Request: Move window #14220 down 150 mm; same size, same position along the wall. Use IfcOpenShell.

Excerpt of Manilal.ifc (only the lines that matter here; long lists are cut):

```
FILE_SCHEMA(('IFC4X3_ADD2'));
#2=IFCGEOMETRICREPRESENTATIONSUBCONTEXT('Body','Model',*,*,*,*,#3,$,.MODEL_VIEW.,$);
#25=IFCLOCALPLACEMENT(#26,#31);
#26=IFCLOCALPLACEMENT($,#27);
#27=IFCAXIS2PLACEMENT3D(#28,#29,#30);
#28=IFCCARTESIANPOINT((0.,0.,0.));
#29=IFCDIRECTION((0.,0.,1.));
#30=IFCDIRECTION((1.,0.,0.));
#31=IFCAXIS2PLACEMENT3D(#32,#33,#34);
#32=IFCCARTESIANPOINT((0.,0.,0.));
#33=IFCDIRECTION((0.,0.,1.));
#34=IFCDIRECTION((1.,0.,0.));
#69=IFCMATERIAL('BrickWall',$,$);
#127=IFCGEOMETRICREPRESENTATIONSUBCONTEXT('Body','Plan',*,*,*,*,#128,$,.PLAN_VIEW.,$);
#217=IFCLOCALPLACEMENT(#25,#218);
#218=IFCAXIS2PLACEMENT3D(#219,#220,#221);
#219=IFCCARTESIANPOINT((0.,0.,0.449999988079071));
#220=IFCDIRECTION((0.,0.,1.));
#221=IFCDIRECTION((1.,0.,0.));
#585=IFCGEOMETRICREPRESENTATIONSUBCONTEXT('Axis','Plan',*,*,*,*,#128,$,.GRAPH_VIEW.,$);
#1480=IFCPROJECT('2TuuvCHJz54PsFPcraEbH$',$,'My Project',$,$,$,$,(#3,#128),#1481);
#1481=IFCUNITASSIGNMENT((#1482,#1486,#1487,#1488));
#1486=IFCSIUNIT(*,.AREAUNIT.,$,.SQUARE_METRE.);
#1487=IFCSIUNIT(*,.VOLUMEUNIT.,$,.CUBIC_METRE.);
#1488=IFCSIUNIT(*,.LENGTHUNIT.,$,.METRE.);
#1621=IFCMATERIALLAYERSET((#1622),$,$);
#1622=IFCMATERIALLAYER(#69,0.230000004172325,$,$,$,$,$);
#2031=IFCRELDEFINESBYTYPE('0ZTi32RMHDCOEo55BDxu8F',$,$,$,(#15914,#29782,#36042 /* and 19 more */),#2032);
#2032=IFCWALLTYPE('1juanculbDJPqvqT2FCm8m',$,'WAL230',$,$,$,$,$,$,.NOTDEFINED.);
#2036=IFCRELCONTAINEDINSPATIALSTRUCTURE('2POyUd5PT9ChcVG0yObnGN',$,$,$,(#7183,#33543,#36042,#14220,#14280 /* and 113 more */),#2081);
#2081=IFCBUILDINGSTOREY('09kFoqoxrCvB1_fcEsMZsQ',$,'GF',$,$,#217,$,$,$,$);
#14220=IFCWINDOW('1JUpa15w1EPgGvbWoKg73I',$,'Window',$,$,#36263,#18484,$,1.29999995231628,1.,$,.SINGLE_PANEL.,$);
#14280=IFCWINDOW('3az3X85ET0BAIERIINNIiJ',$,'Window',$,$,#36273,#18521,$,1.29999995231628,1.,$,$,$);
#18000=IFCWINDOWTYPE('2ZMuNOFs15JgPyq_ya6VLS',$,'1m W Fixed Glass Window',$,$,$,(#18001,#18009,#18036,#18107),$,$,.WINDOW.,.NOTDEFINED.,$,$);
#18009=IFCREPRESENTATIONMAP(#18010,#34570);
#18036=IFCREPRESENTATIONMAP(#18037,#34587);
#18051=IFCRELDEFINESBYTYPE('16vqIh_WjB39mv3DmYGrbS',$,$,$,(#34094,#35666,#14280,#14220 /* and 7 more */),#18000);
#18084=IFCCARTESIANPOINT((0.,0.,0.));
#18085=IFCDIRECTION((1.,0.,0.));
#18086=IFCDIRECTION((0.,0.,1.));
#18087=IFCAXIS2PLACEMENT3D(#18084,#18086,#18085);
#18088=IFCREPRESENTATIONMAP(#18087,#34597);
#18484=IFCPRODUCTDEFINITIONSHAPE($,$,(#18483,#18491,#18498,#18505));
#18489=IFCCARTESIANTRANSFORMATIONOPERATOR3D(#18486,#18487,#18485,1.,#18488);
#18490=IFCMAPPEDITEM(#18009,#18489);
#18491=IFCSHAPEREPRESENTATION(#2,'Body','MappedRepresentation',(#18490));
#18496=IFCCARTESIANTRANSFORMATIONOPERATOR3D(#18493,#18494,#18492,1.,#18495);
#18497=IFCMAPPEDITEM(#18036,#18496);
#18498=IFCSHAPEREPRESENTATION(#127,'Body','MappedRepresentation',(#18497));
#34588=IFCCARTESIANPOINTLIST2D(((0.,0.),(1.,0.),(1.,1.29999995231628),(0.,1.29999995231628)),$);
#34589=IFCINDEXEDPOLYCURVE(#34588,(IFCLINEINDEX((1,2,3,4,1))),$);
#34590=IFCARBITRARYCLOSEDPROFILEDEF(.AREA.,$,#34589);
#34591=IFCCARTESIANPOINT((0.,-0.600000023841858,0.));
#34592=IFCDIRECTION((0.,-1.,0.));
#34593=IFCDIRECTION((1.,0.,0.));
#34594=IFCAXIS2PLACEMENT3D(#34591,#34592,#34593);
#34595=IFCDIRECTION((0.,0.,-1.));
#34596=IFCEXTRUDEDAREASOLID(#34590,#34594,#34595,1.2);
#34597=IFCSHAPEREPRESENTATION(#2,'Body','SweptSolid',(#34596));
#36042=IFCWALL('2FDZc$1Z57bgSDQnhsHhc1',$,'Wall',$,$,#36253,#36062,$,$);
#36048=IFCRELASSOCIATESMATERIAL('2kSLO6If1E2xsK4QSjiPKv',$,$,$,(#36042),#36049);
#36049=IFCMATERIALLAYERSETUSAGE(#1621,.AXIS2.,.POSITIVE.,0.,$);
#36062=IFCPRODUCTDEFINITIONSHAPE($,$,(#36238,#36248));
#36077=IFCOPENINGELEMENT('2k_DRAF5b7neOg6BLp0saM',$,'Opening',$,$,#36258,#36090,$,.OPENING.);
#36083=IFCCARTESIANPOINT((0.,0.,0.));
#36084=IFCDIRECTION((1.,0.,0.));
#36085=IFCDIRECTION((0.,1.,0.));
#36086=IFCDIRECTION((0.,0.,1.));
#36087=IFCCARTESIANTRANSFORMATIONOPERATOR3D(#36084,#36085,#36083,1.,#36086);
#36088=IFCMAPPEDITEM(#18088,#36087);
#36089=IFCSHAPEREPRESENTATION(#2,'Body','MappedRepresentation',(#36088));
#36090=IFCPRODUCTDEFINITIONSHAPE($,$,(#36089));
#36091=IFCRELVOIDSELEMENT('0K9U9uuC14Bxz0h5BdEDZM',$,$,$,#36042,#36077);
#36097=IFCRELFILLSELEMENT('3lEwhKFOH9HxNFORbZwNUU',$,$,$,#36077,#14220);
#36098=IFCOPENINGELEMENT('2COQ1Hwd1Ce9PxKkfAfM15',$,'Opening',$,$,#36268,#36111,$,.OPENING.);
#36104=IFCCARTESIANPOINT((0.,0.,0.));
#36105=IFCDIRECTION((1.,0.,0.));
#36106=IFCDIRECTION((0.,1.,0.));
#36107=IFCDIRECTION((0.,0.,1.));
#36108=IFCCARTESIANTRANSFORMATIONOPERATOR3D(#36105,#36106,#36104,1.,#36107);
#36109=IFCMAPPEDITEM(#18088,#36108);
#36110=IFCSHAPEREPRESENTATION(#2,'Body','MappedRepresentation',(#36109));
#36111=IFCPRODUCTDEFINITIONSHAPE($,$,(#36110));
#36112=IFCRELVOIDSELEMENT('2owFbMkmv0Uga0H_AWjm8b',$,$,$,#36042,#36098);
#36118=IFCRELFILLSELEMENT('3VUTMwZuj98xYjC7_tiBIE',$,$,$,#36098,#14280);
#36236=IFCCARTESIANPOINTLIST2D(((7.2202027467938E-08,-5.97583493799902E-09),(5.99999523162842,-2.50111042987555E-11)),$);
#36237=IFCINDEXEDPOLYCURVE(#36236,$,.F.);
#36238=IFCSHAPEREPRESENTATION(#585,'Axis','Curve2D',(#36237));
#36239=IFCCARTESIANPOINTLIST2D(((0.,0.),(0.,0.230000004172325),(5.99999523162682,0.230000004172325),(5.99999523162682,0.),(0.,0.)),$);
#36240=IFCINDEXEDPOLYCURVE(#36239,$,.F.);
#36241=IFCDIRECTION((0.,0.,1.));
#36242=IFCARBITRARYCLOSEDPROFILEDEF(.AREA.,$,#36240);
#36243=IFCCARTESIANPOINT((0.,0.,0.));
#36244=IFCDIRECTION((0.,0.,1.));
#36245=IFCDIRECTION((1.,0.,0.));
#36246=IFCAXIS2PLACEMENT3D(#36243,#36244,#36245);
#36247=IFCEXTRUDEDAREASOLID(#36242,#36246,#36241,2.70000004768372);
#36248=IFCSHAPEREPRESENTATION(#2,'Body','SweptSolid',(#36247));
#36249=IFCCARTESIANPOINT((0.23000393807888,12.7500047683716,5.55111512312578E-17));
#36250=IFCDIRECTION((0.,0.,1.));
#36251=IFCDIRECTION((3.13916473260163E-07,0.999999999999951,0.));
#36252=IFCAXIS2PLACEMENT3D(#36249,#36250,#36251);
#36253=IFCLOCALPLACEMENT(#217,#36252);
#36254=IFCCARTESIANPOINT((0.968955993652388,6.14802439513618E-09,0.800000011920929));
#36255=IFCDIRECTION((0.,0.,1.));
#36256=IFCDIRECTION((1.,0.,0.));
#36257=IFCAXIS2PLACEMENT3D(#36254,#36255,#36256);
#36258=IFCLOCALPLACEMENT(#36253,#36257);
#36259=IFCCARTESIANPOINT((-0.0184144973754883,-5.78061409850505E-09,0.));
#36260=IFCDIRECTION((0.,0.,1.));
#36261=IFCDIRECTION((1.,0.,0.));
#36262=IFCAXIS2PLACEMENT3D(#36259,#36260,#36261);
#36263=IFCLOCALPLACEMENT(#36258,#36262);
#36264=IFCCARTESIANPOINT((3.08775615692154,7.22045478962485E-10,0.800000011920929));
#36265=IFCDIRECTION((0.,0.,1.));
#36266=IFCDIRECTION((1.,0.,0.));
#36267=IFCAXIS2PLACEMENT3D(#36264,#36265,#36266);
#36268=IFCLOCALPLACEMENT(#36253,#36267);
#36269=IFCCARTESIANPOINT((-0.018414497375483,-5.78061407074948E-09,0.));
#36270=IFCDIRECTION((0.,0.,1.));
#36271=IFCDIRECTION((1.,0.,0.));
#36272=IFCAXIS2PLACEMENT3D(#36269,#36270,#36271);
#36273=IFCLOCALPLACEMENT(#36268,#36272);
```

```python
import numpy as np
import ifcopenshell
import ifcopenshell.api.geometry
import ifcopenshell.util.placement
import ifcopenshell.util.unit

model = ifcopenshell.open("Manilal.ifc")
unit_scale = ifcopenshell.util.unit.calculate_unit_scale(model)

window = model.by_guid("1JUpa15w1EPgGvbWoKg73I")
opening = window.FillsVoids[0].RelatingOpeningElement
dz = -0.15 / unit_scale

shift = np.array([0.0, 0.0, dz])
# The window is placed relative to its opening, so it follows when the opening moves.
matrix = ifcopenshell.util.placement.get_local_placement(opening.ObjectPlacement)
matrix[:3, 3] += shift
ifcopenshell.api.geometry.edit_object_placement(
    model, product=opening, matrix=matrix, is_si=False, should_transform_children=True
)

print(f"moved by {dz * unit_scale:+.3f} m")

model.write("Manilal_rev.ifc")
```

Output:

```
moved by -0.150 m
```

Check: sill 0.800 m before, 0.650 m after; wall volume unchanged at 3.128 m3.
